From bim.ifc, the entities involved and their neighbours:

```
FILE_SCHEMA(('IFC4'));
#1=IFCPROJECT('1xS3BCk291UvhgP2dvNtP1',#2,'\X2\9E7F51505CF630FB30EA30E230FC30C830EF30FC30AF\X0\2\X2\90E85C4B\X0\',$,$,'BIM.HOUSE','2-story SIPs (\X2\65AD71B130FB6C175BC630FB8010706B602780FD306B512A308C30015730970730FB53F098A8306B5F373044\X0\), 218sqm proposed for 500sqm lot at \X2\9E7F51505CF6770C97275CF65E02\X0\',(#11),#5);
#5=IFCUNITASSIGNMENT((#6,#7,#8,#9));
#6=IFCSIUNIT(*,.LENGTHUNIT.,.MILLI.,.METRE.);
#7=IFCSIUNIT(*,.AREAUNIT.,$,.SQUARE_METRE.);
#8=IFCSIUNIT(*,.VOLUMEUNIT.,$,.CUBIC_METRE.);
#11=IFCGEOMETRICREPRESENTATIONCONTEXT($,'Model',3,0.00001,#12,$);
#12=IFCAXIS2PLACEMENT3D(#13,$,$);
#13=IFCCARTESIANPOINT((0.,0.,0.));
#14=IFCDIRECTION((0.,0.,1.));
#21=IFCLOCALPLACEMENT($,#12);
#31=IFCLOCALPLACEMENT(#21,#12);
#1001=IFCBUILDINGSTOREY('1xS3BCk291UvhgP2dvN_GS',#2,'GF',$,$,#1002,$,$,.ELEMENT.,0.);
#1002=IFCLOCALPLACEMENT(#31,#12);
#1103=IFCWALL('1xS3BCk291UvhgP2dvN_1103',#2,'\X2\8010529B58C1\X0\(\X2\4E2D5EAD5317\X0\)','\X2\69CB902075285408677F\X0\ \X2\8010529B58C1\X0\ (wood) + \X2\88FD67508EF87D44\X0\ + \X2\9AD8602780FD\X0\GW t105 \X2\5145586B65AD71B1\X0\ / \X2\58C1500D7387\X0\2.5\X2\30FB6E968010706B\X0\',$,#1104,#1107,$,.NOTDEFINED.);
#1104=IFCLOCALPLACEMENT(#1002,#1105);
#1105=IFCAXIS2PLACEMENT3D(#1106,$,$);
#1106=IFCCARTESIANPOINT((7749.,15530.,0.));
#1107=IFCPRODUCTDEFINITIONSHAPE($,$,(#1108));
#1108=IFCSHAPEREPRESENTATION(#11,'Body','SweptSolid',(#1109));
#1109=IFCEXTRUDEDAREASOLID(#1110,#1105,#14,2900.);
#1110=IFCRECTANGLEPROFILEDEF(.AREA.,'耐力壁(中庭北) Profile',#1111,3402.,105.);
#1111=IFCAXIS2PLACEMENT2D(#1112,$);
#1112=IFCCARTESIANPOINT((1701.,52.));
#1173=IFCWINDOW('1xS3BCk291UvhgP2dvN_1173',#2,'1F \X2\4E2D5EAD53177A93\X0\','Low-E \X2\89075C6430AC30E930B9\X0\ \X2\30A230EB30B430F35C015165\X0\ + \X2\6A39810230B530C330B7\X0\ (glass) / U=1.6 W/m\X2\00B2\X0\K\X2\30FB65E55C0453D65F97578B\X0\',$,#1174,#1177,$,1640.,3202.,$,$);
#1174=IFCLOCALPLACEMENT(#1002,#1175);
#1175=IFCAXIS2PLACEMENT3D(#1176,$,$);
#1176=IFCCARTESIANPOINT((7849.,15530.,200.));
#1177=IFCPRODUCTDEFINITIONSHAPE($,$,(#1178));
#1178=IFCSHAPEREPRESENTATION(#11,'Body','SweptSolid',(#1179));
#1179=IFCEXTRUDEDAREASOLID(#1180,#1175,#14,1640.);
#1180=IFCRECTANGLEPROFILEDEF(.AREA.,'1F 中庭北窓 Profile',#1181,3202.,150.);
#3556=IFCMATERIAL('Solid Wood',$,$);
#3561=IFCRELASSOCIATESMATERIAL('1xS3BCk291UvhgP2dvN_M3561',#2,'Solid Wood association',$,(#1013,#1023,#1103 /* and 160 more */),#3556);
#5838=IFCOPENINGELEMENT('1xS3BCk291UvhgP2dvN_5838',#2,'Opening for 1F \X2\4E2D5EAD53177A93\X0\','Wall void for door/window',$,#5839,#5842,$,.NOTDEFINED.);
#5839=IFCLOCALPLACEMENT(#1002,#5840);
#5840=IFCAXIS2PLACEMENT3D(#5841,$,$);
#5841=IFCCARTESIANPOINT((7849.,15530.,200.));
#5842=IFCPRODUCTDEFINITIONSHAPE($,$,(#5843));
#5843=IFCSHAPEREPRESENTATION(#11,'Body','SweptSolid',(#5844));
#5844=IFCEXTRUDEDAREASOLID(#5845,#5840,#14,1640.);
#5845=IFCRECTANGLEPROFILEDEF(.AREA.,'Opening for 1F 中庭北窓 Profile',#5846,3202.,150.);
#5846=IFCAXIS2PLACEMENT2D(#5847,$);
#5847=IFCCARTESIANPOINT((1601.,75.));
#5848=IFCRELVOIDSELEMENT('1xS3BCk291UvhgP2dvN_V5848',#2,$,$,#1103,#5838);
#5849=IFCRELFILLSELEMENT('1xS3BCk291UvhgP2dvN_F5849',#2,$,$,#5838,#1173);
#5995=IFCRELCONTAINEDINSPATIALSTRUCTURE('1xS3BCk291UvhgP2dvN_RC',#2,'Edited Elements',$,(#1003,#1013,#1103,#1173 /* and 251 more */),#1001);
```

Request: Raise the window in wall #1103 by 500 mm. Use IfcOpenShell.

```python
import numpy as np
import ifcopenshell
import ifcopenshell.api.geometry
import ifcopenshell.util.placement
import ifcopenshell.util.unit

model = ifcopenshell.open("bim.ifc")
unit_scale = ifcopenshell.util.unit.calculate_unit_scale(model)

window = model.by_guid("1xS3BCk291UvhgP2dvN_1173")
opening = window.FillsVoids[0].RelatingOpeningElement
dz = 0.5 / unit_scale

shift = np.array([0.0, 0.0, dz])
# The window is not placed relative to its opening, so move both.
for product in (opening, window):
    matrix = ifcopenshell.util.placement.get_local_placement(product.ObjectPlacement)
    matrix[:3, 3] += shift
    ifcopenshell.api.geometry.edit_object_placement(model, product=product, matrix=matrix, is_si=False)

print(f"moved by {dz * unit_scale:+.3f} m")

model.write("bim_updated.ifc")
```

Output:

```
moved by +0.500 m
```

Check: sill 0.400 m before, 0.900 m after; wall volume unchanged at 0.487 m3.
